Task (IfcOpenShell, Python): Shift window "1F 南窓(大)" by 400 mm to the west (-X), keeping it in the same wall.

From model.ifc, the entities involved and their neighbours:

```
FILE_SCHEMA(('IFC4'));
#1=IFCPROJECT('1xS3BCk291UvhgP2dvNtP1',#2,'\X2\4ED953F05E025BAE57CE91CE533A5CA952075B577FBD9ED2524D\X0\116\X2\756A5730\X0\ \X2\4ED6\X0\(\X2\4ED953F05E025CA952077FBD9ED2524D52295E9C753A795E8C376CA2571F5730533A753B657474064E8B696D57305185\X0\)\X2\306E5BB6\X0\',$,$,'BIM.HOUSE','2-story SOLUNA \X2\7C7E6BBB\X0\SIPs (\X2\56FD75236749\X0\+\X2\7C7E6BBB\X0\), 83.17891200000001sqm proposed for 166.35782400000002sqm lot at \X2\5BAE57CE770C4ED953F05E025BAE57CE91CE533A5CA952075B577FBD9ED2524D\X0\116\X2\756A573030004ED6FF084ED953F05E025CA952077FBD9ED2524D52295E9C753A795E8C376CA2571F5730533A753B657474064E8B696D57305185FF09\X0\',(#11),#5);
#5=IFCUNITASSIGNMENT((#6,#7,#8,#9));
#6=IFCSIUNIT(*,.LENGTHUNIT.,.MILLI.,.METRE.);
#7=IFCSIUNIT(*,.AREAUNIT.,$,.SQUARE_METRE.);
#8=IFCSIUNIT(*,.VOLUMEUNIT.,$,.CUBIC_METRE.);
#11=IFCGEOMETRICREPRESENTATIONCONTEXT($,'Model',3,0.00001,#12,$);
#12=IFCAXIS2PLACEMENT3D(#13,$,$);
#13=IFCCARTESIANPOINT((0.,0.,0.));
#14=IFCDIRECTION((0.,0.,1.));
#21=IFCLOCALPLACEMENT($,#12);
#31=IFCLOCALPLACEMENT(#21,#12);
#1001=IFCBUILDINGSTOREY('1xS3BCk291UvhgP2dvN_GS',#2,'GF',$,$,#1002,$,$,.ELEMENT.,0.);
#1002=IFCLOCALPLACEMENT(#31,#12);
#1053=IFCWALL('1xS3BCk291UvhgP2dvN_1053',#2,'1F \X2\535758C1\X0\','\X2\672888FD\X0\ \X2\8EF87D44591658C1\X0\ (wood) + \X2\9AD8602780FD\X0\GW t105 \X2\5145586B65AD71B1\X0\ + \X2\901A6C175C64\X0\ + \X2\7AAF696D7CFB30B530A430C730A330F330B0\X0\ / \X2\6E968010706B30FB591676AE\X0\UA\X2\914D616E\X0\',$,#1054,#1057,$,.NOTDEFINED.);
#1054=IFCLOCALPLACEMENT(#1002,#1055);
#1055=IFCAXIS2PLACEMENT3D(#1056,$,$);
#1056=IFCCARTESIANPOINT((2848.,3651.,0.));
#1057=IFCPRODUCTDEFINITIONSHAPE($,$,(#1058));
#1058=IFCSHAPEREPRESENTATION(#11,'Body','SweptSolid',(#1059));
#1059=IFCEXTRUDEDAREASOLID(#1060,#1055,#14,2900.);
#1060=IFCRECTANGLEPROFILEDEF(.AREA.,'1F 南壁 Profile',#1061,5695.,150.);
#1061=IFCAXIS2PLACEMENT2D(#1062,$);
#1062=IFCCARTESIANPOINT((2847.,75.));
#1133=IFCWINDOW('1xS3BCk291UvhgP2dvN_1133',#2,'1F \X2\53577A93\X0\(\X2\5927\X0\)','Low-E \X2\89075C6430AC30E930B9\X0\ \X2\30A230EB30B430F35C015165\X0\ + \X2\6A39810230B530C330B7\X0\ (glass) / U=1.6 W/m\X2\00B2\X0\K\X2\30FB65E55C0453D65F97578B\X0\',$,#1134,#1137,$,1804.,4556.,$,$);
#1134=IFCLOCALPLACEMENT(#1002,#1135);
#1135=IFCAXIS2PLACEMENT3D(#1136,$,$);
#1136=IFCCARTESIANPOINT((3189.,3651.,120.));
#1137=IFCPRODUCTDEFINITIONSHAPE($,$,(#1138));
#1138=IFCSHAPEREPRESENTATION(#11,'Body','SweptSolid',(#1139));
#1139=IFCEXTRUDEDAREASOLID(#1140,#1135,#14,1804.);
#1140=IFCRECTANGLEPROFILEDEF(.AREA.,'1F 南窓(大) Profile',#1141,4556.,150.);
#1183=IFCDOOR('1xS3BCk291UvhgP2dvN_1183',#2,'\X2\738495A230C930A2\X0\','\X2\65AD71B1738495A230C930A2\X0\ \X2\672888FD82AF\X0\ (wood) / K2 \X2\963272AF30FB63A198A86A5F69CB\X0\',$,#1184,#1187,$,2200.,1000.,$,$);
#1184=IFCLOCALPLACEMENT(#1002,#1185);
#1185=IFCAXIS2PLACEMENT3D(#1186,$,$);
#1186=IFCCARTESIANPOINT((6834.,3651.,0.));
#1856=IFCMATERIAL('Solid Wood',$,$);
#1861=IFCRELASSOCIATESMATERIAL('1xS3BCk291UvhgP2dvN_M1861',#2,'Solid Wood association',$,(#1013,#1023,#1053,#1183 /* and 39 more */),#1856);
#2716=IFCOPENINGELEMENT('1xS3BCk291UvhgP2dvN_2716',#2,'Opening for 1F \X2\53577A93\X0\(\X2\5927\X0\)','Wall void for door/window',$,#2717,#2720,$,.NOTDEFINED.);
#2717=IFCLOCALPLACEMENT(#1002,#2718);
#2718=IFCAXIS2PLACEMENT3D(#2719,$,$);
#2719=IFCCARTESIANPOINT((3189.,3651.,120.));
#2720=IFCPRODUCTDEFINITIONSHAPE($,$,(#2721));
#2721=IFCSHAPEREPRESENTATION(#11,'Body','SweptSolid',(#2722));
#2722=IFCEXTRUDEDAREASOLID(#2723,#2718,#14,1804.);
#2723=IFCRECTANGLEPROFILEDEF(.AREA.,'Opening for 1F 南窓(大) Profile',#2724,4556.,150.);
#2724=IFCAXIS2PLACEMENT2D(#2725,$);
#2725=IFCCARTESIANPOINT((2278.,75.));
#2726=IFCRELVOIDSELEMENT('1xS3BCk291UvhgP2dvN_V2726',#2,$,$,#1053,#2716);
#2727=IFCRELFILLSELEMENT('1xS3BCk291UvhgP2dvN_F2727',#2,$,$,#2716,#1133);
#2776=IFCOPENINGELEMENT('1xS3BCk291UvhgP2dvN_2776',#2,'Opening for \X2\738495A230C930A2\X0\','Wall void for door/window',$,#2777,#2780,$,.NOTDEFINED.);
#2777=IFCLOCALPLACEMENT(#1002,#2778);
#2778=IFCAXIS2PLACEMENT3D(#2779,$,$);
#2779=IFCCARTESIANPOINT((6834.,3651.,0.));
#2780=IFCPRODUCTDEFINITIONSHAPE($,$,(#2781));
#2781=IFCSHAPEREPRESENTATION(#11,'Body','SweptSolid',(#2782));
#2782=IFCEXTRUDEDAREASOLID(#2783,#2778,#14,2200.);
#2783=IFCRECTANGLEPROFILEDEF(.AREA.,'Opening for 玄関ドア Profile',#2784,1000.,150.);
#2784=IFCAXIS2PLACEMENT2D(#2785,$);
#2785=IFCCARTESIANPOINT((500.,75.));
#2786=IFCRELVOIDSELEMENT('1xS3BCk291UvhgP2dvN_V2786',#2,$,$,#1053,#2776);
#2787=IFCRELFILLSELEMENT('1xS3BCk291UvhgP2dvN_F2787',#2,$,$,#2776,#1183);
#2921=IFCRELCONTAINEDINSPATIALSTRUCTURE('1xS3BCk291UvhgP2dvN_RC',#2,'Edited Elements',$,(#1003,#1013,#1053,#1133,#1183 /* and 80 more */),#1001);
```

```python
import ifcopenshell
import ifcopenshell.api.geometry
import ifcopenshell.util.placement
import ifcopenshell.util.unit

model = ifcopenshell.open("model.ifc")
unit_scale = ifcopenshell.util.unit.calculate_unit_scale(model)

window = model.by_guid("1xS3BCk291UvhgP2dvN_1133")
opening = window.FillsVoids[0].RelatingOpeningElement
wall = opening.VoidsElements[0].RelatingBuildingElement

wall_matrix = ifcopenshell.util.placement.get_local_placement(wall.ObjectPlacement)
shift = wall_matrix[:3, 0] * -0.4 / unit_scale
before = ifcopenshell.util.placement.get_local_placement(window.ObjectPlacement)[:3, 3].copy()

# The window is not placed relative to its opening, so move both.
for product in (opening, window):
    matrix = ifcopenshell.util.placement.get_local_placement(product.ObjectPlacement)
    matrix[:3, 3] += shift
    ifcopenshell.api.geometry.edit_object_placement(model, product=product, matrix=matrix, is_si=False)

after = ifcopenshell.util.placement.get_local_placement(window.ObjectPlacement)[:3, 3]
print("window moved by", (after - before).round(3) + 0.0)

model.write("model_updated.ifc")
```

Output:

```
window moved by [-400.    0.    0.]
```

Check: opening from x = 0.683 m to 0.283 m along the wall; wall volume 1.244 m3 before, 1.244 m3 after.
